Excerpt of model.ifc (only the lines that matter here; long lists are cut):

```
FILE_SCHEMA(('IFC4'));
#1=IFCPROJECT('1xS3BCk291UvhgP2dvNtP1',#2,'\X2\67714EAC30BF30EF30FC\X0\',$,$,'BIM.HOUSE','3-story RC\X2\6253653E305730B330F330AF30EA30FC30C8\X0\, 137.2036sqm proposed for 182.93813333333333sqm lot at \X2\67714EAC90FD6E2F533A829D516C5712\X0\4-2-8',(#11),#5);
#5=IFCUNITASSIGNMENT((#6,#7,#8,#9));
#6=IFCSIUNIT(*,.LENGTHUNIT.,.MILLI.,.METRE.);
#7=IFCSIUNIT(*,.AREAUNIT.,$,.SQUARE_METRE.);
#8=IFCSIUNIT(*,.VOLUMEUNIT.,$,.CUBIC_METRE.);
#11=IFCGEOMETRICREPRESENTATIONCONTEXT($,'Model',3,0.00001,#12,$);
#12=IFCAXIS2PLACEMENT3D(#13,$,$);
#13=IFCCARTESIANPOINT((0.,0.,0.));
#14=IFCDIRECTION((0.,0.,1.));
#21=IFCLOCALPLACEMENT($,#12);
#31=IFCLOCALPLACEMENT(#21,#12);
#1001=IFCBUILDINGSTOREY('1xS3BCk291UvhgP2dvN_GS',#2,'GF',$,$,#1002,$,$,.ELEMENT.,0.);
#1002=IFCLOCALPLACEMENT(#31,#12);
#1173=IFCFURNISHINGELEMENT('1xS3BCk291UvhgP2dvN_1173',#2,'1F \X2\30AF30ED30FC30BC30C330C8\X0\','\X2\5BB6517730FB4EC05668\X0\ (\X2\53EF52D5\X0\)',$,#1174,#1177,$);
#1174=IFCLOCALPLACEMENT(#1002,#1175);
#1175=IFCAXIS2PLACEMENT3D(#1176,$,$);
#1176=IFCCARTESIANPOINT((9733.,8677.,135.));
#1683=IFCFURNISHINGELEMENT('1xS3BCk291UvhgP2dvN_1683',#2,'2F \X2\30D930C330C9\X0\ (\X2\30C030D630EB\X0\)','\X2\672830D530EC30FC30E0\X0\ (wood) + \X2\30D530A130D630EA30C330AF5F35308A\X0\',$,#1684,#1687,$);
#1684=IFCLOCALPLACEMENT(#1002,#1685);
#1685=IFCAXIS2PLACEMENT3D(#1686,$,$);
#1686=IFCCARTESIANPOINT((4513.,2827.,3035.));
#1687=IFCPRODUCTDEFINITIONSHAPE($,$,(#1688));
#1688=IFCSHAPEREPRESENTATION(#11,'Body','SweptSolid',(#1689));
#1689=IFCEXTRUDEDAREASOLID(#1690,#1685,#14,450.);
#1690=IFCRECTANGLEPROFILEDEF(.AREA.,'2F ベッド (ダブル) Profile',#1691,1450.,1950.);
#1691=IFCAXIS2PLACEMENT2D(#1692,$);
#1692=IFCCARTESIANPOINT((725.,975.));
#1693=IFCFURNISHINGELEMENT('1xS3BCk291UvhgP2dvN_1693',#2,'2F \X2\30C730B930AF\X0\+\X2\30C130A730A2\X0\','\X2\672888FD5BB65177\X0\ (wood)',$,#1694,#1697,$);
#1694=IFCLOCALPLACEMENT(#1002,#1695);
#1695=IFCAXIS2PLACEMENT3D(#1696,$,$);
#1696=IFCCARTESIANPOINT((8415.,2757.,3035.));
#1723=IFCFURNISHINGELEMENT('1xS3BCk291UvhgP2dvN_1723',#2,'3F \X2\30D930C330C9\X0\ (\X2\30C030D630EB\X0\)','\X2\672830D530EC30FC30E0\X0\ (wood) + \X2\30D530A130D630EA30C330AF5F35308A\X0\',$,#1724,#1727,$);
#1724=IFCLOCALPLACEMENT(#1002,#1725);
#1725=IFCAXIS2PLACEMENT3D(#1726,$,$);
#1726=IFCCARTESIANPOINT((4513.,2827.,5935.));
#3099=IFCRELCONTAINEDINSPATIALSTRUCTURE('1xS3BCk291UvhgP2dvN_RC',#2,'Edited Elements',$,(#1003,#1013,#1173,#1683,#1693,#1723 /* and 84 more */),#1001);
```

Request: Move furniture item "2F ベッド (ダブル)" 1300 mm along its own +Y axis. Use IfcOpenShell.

```python
import ifcopenshell
import ifcopenshell.api.geometry
import ifcopenshell.util.placement
import ifcopenshell.util.unit

model = ifcopenshell.open("model.ifc")
unit_scale = ifcopenshell.util.unit.calculate_unit_scale(model)

item = model.by_guid("1xS3BCk291UvhgP2dvN_1683")
matrix = ifcopenshell.util.placement.get_local_placement(item.ObjectPlacement)
matrix[:3, 3] += matrix[:3, 1] * 1.3 / unit_scale
ifcopenshell.api.geometry.edit_object_placement(model, product=item, matrix=matrix, is_si=False)

print(ifcopenshell.util.placement.get_local_placement(item.ObjectPlacement).round(3) + 0.0)

model.write("model-out.ifc")
```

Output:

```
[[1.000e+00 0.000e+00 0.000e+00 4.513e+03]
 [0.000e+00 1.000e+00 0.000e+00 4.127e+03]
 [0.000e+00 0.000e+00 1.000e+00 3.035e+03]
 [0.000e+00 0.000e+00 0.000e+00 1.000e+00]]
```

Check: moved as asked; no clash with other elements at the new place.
